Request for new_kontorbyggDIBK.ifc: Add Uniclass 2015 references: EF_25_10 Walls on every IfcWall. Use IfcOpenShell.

First a look at what the model holds.

```python
import ifcopenshell

model = ifcopenshell.open("new_kontorbyggDIBK.ifc")
print(model.schema)
print("classifications:", [c.Name for c in model.by_type("IfcClassification")])
for ifc_class in ("IfcDoor", "IfcRoof", "IfcStair", "IfcWall", "IfcWindow"):
    print(ifc_class, len(model.by_type(ifc_class)))
```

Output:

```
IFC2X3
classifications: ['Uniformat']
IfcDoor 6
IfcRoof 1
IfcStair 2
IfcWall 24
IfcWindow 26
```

```python
import ifcopenshell
import ifcopenshell.api.classification

model = ifcopenshell.open("new_kontorbyggDIBK.ifc")

# IFC2X3 requires Source and Edition and has no link from the project to the system.
system = model.create_entity("IfcClassification", Source="NBS", Edition="2015", Name="Uniclass 2015")

codes = {
    "IfcWall": ("EF_25_10", "Walls"),
}
for ifc_class, (code, name) in codes.items():
    products = model.by_type(ifc_class)
    ifcopenshell.api.classification.add_reference(
        model, products=products, classification=system, identification=code, name=name
    )
    print(code, len(products))

model.write("new_kontorbyggDIBK_rev.ifc")
```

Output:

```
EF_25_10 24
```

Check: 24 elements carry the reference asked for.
